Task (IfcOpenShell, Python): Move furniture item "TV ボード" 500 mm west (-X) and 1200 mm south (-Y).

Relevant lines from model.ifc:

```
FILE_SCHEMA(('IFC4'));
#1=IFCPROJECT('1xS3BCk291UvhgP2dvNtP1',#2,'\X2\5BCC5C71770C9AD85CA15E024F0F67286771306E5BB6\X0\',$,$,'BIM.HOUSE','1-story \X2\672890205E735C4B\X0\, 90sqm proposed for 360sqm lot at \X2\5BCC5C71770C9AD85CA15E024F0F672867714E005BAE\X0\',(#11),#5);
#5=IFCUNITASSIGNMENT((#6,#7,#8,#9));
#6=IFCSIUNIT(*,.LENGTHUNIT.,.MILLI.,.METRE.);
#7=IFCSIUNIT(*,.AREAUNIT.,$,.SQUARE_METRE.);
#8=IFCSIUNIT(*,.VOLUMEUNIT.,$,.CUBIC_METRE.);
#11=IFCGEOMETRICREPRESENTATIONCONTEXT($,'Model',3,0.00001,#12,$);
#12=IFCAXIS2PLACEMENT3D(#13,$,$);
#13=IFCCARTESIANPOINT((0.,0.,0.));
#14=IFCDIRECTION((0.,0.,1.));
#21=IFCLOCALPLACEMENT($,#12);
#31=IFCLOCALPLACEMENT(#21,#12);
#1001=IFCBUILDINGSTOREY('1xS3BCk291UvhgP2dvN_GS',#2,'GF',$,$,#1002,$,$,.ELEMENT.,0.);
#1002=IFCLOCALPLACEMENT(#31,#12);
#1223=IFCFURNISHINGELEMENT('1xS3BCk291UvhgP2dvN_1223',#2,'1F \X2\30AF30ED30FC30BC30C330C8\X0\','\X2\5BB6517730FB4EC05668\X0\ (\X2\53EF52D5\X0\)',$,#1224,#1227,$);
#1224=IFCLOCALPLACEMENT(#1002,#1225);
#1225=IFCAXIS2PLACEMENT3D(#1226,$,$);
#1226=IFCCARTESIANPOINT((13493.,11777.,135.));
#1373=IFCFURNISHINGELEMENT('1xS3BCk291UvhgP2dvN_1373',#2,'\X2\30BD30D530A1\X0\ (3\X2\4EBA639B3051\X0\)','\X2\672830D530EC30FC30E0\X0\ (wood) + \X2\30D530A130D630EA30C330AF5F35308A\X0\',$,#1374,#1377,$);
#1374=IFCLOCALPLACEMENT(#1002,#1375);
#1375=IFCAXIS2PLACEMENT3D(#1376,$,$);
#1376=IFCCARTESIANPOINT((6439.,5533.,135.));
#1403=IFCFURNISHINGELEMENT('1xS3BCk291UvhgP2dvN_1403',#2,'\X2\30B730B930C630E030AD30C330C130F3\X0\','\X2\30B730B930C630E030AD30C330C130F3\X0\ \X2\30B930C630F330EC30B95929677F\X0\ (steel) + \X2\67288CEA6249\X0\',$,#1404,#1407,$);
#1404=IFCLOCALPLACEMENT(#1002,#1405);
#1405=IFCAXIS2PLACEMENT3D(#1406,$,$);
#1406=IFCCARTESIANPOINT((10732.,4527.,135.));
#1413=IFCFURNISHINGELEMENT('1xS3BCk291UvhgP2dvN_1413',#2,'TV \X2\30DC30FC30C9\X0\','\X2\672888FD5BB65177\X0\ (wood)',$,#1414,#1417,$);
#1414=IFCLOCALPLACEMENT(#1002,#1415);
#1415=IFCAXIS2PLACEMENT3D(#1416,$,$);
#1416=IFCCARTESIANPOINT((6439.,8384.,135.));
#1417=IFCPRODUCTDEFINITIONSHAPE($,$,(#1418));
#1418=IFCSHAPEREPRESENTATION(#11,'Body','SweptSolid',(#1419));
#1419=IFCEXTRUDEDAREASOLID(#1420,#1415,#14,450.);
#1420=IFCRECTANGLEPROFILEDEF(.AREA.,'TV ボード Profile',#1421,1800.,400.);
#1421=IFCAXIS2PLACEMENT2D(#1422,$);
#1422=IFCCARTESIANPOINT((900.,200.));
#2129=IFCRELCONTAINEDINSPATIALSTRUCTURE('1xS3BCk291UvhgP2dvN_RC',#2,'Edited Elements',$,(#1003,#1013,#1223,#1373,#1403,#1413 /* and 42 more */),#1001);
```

```python
import ifcopenshell
import ifcopenshell.api.geometry
import ifcopenshell.util.placement
import ifcopenshell.util.unit

model = ifcopenshell.open("model.ifc")
unit_scale = ifcopenshell.util.unit.calculate_unit_scale(model)

item = model.by_guid("1xS3BCk291UvhgP2dvN_1413")
matrix = ifcopenshell.util.placement.get_local_placement(item.ObjectPlacement)
matrix[0, 3] -= 0.5 / unit_scale
matrix[1, 3] -= 1.2 / unit_scale
ifcopenshell.api.geometry.edit_object_placement(model, product=item, matrix=matrix, is_si=False)

print(ifcopenshell.util.placement.get_local_placement(item.ObjectPlacement).round(3) + 0.0)

model.write("model_updated.ifc")
```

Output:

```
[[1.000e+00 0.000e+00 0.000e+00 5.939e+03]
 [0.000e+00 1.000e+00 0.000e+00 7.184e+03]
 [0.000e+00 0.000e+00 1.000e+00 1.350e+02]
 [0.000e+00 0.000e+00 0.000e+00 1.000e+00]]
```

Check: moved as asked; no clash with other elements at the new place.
